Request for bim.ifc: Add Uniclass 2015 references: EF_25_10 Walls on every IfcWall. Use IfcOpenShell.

First a look at what the model holds.

```python
import ifcopenshell

model = ifcopenshell.open("bim.ifc")
print(model.schema)
print("classifications:", [c.Name for c in model.by_type("IfcClassification")])
for ifc_class in ("IfcDoor", "IfcRoof", "IfcStair", "IfcWall", "IfcWindow"):
    print(ifc_class, len(model.by_type(ifc_class)))
```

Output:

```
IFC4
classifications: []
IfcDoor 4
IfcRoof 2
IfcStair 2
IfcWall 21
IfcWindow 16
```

```python
import ifcopenshell
import ifcopenshell.api.classification

model = ifcopenshell.open("bim.ifc")

system = ifcopenshell.api.classification.add_classification(model, classification="Uniclass 2015")

codes = {
    "IfcWall": ("EF_25_10", "Walls"),
}
for ifc_class, (code, name) in codes.items():
    products = model.by_type(ifc_class)
    ifcopenshell.api.classification.add_reference(
        model, products=products, classification=system, identification=code, name=name
    )
    print(code, len(products))

model.write("bim_rev.ifc")
```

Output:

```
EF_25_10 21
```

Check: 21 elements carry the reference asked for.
